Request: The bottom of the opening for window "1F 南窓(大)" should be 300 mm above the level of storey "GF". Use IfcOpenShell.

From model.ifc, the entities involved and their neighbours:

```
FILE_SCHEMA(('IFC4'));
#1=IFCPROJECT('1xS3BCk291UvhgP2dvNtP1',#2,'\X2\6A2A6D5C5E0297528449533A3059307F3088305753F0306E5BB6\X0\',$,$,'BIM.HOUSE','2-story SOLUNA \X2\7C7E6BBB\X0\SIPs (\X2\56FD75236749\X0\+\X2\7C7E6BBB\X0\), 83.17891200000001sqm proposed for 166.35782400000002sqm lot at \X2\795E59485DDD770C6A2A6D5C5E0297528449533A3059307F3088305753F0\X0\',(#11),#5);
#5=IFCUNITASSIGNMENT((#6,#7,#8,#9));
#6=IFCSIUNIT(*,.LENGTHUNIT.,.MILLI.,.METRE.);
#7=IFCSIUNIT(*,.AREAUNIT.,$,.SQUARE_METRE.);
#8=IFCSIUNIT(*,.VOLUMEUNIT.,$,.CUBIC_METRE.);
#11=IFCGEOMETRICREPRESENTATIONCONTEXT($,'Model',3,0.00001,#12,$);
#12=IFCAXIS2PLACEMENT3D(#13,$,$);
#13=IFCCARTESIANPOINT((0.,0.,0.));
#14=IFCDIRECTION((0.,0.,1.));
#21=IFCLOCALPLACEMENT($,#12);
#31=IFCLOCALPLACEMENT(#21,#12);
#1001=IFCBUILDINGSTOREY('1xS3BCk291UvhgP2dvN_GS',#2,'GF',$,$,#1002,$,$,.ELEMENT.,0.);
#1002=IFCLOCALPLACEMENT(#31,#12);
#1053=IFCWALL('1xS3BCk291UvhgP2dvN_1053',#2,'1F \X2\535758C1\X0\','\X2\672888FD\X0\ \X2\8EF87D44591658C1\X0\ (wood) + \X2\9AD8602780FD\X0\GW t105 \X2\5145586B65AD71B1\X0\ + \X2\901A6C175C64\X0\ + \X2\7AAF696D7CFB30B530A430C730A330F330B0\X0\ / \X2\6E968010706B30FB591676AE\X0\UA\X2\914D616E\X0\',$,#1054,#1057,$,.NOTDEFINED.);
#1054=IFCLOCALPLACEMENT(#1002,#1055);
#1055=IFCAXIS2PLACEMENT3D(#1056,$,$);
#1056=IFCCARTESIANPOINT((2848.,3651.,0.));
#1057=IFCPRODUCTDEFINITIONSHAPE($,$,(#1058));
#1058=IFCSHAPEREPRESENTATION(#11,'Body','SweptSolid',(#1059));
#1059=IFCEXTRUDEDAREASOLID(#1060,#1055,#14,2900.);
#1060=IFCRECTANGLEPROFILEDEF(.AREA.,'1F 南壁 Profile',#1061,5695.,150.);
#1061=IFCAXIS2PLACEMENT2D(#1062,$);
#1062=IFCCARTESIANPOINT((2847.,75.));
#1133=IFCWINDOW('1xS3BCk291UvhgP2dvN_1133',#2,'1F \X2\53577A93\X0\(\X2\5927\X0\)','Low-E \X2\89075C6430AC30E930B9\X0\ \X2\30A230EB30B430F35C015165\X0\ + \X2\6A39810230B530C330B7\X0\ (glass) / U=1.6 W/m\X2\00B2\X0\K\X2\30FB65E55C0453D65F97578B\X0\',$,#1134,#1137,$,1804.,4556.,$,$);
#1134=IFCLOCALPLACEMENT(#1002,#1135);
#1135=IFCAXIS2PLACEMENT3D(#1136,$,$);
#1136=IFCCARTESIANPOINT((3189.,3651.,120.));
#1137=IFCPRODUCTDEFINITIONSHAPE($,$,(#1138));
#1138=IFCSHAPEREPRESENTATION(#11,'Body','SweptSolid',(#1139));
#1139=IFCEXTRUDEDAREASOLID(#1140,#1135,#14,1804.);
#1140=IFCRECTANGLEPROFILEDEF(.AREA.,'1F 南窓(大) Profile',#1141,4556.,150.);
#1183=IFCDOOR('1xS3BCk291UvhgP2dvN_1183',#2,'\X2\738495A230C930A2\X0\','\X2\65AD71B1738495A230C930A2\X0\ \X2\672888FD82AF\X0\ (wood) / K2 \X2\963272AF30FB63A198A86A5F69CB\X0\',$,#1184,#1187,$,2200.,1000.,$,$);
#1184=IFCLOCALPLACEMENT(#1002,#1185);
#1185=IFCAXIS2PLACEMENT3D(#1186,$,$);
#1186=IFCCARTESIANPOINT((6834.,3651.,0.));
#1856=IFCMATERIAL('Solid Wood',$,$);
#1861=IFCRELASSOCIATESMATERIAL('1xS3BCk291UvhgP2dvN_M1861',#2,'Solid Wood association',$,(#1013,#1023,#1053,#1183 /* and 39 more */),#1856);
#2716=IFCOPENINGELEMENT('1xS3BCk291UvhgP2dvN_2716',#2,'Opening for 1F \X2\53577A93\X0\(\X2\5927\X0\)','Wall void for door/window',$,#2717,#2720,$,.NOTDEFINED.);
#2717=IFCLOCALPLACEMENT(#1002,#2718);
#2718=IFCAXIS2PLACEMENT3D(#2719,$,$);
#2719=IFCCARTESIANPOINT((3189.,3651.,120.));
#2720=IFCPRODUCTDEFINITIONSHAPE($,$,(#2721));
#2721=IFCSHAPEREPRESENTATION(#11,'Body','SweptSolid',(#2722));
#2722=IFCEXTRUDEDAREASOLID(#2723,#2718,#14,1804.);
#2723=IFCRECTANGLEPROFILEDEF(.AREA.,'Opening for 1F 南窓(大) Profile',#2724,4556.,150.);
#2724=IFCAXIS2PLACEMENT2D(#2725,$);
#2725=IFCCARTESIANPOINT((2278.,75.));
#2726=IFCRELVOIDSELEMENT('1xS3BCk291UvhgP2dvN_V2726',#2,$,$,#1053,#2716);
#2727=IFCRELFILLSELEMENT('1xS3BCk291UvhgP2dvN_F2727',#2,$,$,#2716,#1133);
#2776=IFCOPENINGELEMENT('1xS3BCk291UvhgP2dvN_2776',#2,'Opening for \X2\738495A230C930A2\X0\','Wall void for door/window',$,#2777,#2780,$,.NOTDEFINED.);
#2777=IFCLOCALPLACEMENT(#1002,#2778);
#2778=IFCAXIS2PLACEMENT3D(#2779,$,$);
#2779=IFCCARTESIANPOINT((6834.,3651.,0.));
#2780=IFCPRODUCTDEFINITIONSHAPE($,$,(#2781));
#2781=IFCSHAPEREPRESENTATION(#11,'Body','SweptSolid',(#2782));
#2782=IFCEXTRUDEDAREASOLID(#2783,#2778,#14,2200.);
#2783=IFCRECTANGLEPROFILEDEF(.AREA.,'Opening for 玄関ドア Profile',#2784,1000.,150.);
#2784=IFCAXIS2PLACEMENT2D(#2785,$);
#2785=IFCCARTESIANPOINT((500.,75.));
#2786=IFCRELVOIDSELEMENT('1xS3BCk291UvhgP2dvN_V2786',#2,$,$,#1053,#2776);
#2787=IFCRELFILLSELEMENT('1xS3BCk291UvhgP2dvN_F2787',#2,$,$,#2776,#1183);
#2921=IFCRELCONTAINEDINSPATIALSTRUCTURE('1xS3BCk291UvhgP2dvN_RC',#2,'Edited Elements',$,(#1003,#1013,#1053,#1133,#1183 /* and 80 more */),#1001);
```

```python
import numpy as np
import ifcopenshell
import ifcopenshell.api.geometry
import ifcopenshell.geom
import ifcopenshell.util.element
import ifcopenshell.util.placement
import ifcopenshell.util.shape
import ifcopenshell.util.unit

model = ifcopenshell.open("model.ifc")
unit_scale = ifcopenshell.util.unit.calculate_unit_scale(model)

window = model.by_guid("1xS3BCk291UvhgP2dvN_1133")
opening = window.FillsVoids[0].RelatingOpeningElement
storey = ifcopenshell.util.element.get_container(window, ifc_class="IfcBuildingStorey")
level = ifcopenshell.util.placement.get_local_placement(storey.ObjectPlacement)[2, 3]

# The opening's origin need not be at the sill, so measure its lowest point.
shape = ifcopenshell.geom.create_shape(ifcopenshell.geom.settings(), opening)
bottom = ifcopenshell.util.shape.get_shape_bottom_elevation(shape, shape.geometry) / unit_scale
dz = level + 300.0 - bottom

shift = np.array([0.0, 0.0, dz])
# The window is not placed relative to its opening, so move both.
for product in (opening, window):
    matrix = ifcopenshell.util.placement.get_local_placement(product.ObjectPlacement)
    matrix[:3, 3] += shift
    ifcopenshell.api.geometry.edit_object_placement(model, product=product, matrix=matrix, is_si=False)

print(f"moved by {dz * unit_scale:+.3f} m")

model.write("model_rev.ifc")
```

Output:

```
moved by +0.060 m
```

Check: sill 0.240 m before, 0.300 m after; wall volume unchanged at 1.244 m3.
